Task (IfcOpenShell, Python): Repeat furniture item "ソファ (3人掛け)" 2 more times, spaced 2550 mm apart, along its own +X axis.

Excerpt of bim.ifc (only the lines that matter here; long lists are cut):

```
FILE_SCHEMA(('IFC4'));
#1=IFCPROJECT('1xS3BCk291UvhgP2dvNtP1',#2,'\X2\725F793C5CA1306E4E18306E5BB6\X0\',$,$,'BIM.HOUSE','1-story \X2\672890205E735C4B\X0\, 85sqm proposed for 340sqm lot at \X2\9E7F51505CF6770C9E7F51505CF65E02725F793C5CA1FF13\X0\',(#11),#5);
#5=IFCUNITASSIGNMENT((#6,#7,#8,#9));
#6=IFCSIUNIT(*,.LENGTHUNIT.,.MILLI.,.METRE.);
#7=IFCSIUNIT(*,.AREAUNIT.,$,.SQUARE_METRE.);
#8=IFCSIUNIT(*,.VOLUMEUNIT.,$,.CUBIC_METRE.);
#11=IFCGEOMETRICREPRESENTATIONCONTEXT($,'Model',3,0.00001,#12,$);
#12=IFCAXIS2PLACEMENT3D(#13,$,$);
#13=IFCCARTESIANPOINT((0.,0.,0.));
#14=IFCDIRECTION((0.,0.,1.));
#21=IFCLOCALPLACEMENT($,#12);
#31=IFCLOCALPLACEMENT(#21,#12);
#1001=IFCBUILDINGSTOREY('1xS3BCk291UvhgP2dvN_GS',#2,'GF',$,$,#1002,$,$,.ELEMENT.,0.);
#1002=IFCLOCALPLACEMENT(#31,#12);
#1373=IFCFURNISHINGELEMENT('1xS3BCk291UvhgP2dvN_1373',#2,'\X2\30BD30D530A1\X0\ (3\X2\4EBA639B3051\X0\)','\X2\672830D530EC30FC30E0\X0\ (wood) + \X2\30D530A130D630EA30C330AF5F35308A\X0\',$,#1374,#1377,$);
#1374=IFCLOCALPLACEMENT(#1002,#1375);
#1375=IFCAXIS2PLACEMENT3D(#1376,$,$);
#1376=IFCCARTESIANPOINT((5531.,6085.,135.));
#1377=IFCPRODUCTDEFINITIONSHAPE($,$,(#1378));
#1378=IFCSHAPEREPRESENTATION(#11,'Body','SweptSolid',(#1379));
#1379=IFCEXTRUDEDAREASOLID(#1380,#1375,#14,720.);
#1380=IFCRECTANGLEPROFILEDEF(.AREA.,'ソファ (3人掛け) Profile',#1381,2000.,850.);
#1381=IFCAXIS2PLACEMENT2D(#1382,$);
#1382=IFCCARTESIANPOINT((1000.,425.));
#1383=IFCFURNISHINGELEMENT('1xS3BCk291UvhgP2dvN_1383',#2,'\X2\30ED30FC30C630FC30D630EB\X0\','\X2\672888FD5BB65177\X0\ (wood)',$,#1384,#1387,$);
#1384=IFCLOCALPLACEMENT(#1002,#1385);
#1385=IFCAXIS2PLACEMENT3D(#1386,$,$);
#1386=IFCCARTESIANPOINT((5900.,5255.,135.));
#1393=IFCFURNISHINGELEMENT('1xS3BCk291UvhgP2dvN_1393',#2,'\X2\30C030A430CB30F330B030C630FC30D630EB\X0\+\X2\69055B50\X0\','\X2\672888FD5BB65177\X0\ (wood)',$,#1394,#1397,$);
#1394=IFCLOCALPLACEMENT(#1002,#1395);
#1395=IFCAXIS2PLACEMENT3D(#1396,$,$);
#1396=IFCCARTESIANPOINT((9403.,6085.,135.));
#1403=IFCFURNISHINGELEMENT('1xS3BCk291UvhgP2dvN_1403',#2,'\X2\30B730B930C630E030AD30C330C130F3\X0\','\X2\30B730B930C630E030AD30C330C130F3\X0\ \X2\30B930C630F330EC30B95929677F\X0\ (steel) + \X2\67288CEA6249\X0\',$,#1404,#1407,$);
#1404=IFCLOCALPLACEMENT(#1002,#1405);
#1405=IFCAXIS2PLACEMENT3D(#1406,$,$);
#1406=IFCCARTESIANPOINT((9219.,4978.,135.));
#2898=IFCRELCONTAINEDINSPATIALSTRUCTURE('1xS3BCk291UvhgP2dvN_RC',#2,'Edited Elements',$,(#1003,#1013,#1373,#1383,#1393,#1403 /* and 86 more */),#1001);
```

```python
import ifcopenshell
import ifcopenshell.api.geometry
import ifcopenshell.api.root
import ifcopenshell.util.element
import ifcopenshell.util.placement
import ifcopenshell.util.unit

model = ifcopenshell.open("bim.ifc")
unit_scale = ifcopenshell.util.unit.calculate_unit_scale(model)


def reuse_history(source, copy):
    """copy_class also copies each property set's owner history, people and application; keep the originals."""
    for rel in copy.IsDefinedBy:
        if rel.is_a("IfcRelDefinesByProperties") and (history := rel.RelatingPropertyDefinition.OwnerHistory):
            rel.RelatingPropertyDefinition.OwnerHistory = source.OwnerHistory
            ifcopenshell.util.element.remove_deep2(model, history)


source = model.by_guid("1xS3BCk291UvhgP2dvN_1373")
base = ifcopenshell.util.placement.get_local_placement(source.ObjectPlacement)
step = base[:3, 0] * 2.55 / unit_scale

for i in range(1, 3):
    copy = ifcopenshell.api.root.copy_class(model, product=source)
    copy.Representation = ifcopenshell.util.element.copy_deep(
        model, source.Representation, exclude=["IfcGeometricRepresentationContext", "IfcRepresentationMap"]
    )
    reuse_history(source, copy)
    matrix = base.copy()
    matrix[:3, 3] += i * step
    print("added at", matrix[:3, 3].round(3) + 0.0)
    ifcopenshell.api.geometry.edit_object_placement(model, product=copy, matrix=matrix, is_si=False)

model.write("bim_updated.ifc")
```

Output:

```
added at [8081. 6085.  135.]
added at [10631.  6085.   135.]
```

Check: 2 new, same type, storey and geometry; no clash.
